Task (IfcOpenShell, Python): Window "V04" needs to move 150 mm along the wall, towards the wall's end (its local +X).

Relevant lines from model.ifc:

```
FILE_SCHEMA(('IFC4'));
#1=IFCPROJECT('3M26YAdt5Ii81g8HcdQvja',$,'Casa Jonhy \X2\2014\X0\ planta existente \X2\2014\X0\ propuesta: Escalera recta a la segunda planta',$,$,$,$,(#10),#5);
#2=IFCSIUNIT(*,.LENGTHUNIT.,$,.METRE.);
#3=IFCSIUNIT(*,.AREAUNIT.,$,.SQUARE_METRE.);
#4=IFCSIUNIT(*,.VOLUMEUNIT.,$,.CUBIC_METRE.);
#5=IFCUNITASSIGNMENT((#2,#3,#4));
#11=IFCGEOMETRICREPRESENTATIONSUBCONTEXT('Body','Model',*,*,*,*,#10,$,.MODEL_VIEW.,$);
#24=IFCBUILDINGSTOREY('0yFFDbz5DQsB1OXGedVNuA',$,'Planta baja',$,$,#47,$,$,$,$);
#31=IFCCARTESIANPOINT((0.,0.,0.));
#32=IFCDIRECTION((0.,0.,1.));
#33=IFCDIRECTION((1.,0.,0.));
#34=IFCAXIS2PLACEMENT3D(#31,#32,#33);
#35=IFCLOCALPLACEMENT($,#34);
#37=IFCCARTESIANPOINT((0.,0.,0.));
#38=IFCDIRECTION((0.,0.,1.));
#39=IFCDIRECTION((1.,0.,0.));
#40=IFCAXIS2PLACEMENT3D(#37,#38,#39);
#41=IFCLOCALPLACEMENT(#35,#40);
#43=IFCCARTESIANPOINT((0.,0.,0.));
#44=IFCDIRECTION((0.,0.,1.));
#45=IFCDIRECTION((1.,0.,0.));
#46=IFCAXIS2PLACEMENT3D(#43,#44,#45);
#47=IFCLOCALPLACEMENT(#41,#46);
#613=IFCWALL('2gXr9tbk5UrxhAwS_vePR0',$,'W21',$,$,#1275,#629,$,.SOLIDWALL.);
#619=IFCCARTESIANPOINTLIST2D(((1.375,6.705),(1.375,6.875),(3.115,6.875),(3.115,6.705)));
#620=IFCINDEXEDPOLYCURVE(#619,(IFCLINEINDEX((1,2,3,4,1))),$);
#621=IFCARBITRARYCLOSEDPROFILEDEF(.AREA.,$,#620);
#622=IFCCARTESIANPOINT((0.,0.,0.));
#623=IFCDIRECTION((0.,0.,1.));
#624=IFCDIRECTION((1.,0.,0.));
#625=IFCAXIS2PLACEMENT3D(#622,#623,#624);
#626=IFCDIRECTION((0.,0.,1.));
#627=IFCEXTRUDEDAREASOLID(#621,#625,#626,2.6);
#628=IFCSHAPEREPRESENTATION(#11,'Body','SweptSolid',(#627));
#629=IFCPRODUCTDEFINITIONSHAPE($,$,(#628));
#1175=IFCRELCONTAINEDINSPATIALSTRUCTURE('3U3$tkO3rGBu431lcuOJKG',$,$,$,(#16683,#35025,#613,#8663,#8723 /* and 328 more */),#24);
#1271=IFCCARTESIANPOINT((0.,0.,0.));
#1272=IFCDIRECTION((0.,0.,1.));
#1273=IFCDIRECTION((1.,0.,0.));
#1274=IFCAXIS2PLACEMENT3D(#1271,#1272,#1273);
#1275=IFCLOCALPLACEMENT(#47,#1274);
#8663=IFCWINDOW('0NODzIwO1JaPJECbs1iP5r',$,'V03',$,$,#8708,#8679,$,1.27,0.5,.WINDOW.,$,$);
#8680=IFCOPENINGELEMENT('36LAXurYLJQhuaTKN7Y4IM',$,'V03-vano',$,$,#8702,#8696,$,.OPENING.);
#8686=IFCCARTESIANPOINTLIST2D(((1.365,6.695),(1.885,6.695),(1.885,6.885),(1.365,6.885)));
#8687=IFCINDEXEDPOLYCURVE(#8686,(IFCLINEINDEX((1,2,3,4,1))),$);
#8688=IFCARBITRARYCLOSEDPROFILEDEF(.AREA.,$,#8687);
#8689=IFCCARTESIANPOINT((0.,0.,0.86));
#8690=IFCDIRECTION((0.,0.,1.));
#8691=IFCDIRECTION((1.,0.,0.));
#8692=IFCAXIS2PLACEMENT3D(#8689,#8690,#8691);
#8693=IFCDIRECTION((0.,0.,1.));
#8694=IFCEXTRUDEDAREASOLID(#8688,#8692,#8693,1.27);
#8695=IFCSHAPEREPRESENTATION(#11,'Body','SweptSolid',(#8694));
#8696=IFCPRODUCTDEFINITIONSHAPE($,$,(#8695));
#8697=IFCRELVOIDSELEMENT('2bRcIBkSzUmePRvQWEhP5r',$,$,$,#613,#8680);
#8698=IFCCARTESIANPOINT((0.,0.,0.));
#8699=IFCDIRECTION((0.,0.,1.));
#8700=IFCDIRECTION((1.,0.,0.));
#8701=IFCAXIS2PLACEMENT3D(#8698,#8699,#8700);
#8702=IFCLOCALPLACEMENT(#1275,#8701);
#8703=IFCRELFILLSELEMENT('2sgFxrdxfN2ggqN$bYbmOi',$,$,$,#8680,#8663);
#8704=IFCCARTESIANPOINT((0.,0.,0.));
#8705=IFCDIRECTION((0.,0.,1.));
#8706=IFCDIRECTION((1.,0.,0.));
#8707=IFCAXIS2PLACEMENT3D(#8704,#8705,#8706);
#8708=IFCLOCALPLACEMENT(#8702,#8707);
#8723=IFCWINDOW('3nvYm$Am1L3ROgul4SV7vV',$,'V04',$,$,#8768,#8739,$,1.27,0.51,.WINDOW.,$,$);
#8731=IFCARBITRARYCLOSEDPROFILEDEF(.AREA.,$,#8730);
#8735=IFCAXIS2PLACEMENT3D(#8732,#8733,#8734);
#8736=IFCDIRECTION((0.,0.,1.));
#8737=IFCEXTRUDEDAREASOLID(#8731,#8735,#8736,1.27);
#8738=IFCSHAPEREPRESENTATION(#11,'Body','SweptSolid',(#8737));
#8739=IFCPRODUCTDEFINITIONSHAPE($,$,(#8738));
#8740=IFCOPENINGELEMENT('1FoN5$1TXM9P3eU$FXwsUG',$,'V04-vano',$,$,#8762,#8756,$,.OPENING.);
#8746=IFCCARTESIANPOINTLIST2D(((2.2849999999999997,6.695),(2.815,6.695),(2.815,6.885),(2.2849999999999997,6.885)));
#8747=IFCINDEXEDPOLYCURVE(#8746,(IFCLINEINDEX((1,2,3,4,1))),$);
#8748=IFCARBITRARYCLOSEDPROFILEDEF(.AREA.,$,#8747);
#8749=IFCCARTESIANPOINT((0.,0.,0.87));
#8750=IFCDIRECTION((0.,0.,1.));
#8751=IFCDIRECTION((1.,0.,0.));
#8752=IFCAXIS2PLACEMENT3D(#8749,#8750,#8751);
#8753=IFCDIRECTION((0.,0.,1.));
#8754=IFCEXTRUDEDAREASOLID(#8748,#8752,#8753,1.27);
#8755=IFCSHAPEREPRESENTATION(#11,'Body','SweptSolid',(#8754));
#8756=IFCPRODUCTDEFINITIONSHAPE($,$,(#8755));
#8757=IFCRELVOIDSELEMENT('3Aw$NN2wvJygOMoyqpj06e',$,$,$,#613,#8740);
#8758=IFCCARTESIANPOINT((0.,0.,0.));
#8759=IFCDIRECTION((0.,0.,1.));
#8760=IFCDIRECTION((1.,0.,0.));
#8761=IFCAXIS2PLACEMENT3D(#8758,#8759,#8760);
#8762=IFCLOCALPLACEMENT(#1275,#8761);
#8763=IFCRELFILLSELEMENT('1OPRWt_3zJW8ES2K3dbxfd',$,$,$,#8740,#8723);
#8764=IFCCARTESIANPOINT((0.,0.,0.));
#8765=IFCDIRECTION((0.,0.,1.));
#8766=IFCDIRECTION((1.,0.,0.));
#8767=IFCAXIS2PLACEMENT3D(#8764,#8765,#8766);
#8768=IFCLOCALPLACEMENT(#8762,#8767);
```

```python
import ifcopenshell
import ifcopenshell.api.geometry
import ifcopenshell.util.placement

model = ifcopenshell.open("model.ifc")

window = model.by_guid("3nvYm$Am1L3ROgul4SV7vV")
opening = window.FillsVoids[0].RelatingOpeningElement
wall = opening.VoidsElements[0].RelatingBuildingElement

wall_matrix = ifcopenshell.util.placement.get_local_placement(wall.ObjectPlacement)
shift = wall_matrix[:3, 0] * 0.15
before = ifcopenshell.util.placement.get_local_placement(window.ObjectPlacement)[:3, 3].copy()

# The window is placed relative to its opening, so it follows when the opening moves.
matrix = ifcopenshell.util.placement.get_local_placement(opening.ObjectPlacement)
matrix[:3, 3] += shift
ifcopenshell.api.geometry.edit_object_placement(
    model, product=opening, matrix=matrix, is_si=False, should_transform_children=True
)

after = ifcopenshell.util.placement.get_local_placement(window.ObjectPlacement)[:3, 3]
print("window moved by", (after - before).round(3) + 0.0)

model.write("model_updated.ifc")
```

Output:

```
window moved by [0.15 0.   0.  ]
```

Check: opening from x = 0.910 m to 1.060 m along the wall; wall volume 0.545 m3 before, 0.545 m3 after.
